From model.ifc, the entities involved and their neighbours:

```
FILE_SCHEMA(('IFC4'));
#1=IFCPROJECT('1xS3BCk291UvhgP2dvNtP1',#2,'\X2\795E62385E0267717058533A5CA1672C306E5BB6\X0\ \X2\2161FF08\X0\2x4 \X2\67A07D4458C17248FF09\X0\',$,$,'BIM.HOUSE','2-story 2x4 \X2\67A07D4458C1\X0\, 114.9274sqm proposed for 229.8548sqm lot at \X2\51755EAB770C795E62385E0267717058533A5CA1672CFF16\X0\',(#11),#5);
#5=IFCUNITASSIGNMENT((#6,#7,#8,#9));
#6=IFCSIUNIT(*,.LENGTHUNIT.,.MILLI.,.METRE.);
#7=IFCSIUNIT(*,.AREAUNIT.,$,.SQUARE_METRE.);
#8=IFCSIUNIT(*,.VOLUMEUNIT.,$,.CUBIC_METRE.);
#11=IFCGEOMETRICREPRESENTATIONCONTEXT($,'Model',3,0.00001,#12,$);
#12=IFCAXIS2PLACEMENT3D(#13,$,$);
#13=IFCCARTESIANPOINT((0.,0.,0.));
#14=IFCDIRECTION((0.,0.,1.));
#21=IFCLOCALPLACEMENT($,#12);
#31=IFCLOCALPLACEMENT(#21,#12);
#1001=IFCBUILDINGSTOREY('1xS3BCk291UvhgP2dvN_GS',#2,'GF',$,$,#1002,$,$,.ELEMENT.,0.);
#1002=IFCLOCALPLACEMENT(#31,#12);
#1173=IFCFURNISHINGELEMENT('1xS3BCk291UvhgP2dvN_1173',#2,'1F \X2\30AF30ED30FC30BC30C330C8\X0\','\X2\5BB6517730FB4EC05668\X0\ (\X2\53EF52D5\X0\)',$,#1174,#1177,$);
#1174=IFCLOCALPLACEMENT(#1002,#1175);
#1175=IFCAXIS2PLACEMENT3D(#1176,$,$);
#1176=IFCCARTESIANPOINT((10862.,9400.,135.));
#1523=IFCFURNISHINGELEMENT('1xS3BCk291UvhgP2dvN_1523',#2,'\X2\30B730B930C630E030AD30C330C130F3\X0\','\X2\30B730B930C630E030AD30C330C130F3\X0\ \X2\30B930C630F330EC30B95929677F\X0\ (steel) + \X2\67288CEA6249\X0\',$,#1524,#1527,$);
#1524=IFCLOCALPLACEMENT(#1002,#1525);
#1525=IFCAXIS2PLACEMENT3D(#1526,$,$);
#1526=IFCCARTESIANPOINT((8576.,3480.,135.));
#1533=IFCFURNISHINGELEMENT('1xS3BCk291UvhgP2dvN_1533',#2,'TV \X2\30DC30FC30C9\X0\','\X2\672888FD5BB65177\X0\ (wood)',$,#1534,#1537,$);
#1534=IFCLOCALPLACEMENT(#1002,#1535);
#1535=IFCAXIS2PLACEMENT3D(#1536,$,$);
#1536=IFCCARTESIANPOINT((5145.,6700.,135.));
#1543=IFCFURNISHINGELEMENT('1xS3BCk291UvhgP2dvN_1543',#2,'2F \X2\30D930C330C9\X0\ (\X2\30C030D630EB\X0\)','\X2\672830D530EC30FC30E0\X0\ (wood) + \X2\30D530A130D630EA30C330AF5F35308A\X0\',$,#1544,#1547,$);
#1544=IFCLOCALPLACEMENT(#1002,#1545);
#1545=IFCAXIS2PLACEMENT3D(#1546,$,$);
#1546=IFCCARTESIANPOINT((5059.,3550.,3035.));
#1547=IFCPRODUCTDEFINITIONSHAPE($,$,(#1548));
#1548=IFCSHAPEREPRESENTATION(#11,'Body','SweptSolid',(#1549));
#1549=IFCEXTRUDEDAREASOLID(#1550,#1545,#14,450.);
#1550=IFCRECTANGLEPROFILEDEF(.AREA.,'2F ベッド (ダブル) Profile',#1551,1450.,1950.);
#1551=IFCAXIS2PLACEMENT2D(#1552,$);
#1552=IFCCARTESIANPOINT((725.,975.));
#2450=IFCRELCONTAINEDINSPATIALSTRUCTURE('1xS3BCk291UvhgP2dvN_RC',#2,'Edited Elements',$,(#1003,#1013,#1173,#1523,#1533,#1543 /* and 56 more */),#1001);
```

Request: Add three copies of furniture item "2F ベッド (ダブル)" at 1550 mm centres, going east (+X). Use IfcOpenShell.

```python
import numpy as np
import ifcopenshell
import ifcopenshell.api.geometry
import ifcopenshell.api.root
import ifcopenshell.util.element
import ifcopenshell.util.placement
import ifcopenshell.util.unit

model = ifcopenshell.open("model.ifc")
unit_scale = ifcopenshell.util.unit.calculate_unit_scale(model)


def reuse_history(source, copy):
    """copy_class also copies each property set's owner history, people and application; keep the originals."""
    for rel in copy.IsDefinedBy:
        if rel.is_a("IfcRelDefinesByProperties") and (history := rel.RelatingPropertyDefinition.OwnerHistory):
            rel.RelatingPropertyDefinition.OwnerHistory = source.OwnerHistory
            ifcopenshell.util.element.remove_deep2(model, history)


source = model.by_id(1543)
base = ifcopenshell.util.placement.get_local_placement(source.ObjectPlacement)
step = np.array([1.0, 0.0, 0.0]) * 1.55 / unit_scale

for i in range(1, 4):
    copy = ifcopenshell.api.root.copy_class(model, product=source)
    copy.Representation = ifcopenshell.util.element.copy_deep(
        model, source.Representation, exclude=["IfcGeometricRepresentationContext", "IfcRepresentationMap"]
    )
    reuse_history(source, copy)
    matrix = base.copy()
    matrix[:3, 3] += i * step
    print("added at", matrix[:3, 3].round(3) + 0.0)
    ifcopenshell.api.geometry.edit_object_placement(model, product=copy, matrix=matrix, is_si=False)

model.write("model_edited.ifc")
```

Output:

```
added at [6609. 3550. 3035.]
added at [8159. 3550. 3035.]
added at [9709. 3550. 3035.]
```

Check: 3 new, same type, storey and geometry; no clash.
